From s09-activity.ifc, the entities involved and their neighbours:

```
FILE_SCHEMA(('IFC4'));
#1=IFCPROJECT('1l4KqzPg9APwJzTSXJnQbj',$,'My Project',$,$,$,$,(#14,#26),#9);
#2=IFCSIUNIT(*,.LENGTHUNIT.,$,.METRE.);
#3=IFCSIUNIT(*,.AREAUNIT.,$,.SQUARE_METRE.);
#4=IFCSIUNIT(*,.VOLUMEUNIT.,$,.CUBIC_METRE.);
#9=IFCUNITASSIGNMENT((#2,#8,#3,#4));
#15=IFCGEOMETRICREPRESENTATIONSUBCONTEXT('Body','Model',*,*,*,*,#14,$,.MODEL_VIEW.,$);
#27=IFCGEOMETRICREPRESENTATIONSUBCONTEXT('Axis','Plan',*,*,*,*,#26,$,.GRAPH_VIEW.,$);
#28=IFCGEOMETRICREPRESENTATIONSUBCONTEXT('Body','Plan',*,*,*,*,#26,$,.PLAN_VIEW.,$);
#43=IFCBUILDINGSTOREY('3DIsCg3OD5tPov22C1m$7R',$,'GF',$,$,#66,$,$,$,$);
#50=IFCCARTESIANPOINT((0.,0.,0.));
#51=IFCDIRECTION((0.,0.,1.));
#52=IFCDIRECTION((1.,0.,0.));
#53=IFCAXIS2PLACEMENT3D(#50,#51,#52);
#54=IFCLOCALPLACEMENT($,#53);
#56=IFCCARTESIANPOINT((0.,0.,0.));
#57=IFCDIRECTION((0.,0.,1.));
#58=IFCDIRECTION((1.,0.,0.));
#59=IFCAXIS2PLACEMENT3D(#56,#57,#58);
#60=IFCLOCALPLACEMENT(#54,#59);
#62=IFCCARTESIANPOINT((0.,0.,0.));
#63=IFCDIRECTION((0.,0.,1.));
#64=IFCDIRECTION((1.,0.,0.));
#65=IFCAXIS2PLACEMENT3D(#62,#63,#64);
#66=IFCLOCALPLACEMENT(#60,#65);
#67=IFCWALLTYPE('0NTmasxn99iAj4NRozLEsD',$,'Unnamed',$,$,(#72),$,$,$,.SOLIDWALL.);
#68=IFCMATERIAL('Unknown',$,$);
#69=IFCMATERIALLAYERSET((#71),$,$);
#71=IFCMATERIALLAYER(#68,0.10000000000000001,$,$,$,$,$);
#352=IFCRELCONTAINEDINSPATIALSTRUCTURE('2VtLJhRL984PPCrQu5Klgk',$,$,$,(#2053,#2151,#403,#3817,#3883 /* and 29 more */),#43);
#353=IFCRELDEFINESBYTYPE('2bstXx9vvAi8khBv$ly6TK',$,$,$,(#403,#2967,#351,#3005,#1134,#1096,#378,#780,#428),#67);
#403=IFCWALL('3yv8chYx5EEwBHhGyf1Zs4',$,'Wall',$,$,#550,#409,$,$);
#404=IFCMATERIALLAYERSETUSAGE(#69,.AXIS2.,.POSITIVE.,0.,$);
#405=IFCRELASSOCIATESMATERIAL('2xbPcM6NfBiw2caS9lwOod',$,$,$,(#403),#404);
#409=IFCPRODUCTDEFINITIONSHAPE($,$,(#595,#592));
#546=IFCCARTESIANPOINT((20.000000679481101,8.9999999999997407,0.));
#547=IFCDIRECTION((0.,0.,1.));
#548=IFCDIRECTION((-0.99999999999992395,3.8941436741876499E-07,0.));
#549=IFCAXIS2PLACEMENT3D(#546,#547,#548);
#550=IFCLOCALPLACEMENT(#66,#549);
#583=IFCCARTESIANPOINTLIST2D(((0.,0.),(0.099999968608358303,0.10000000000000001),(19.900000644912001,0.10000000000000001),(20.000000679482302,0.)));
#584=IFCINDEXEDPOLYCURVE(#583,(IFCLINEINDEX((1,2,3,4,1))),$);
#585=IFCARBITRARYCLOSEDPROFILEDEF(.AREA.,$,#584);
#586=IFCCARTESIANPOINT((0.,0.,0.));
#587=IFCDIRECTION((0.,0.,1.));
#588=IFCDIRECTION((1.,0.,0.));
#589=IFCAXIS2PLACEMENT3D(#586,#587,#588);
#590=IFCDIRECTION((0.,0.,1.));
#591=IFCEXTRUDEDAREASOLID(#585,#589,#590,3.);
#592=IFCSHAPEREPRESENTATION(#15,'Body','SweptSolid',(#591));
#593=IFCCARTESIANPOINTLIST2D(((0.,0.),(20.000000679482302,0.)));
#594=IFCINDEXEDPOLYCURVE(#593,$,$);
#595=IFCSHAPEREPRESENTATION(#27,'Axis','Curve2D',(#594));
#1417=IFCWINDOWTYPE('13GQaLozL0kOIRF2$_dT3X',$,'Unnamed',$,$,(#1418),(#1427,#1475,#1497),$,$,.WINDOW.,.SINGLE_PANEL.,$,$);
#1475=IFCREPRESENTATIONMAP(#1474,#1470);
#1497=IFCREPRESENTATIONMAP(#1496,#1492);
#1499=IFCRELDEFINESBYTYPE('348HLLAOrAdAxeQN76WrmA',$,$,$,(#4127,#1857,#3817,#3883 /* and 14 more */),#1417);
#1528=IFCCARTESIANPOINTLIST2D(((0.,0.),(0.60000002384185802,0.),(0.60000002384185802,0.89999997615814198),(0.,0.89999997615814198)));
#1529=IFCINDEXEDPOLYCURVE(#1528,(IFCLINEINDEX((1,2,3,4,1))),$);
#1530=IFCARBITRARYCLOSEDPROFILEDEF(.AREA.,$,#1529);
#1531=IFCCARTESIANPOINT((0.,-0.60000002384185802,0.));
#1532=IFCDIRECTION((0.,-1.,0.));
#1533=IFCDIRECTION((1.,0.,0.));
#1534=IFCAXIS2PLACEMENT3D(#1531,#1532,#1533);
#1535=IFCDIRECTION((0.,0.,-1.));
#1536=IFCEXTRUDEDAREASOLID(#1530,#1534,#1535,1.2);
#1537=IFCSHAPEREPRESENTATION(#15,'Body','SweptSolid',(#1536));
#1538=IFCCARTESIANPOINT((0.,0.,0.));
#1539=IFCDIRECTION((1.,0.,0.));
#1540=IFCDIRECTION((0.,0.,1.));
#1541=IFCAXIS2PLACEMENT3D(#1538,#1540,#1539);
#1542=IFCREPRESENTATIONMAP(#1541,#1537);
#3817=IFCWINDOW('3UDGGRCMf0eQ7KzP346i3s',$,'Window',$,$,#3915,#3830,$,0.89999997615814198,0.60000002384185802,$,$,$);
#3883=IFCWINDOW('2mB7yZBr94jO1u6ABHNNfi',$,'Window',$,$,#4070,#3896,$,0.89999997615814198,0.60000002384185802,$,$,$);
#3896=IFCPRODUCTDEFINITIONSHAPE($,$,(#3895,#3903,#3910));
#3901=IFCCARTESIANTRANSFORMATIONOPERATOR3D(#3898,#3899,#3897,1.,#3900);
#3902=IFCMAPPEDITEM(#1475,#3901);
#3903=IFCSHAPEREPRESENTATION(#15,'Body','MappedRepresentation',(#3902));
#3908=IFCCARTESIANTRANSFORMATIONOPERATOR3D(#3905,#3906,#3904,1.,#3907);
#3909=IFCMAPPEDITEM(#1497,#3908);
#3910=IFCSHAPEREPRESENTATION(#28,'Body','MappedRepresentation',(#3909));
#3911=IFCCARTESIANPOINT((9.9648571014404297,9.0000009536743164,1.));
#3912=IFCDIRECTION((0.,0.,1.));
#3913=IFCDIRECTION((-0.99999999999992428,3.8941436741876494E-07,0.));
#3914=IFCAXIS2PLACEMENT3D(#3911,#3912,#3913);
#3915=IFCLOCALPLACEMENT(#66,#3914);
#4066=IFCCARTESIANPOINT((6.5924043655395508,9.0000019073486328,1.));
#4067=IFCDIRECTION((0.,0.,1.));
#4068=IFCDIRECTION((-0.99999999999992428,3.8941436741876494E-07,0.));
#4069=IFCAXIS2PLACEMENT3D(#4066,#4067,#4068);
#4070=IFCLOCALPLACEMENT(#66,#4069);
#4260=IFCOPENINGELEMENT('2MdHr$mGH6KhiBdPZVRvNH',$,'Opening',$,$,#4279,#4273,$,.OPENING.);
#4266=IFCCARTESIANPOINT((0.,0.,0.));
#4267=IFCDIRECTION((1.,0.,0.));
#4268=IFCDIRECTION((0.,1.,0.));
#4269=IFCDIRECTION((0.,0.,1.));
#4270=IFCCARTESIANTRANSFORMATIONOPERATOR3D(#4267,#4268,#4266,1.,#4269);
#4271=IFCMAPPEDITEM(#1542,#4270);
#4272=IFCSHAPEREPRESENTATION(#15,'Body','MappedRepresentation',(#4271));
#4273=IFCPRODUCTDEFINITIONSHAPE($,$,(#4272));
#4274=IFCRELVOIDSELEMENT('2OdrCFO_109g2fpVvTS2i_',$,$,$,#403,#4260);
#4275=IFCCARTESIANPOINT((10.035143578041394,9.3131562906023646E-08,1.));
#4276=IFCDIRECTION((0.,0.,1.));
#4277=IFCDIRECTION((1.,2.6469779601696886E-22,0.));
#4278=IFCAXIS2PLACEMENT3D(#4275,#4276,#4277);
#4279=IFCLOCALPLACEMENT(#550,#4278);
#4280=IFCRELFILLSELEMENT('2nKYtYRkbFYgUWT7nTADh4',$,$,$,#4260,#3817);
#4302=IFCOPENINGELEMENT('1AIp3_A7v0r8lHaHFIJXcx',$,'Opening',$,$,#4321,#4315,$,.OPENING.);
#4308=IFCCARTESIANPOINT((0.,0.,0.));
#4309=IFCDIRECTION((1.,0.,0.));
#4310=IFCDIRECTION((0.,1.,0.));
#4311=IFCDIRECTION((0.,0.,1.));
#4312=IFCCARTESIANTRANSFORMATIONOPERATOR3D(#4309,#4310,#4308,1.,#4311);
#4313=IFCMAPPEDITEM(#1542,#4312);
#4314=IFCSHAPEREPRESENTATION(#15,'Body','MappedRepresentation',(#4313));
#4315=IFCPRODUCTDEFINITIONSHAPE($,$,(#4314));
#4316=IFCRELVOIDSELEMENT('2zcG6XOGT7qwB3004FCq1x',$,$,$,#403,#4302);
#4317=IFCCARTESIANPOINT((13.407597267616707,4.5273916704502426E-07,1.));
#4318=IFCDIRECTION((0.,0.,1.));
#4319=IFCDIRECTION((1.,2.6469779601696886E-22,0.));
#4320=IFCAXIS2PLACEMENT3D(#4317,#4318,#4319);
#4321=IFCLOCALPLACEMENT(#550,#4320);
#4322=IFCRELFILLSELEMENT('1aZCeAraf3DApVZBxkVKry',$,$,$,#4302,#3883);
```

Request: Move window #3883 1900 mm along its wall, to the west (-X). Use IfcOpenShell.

```python
import ifcopenshell
import ifcopenshell.api.geometry
import ifcopenshell.util.placement

model = ifcopenshell.open("s09-activity.ifc")

window = model.by_guid("2mB7yZBr94jO1u6ABHNNfi")
opening = window.FillsVoids[0].RelatingOpeningElement
wall = opening.VoidsElements[0].RelatingBuildingElement

wall_matrix = ifcopenshell.util.placement.get_local_placement(wall.ObjectPlacement)
shift = wall_matrix[:3, 0] * 1.9
before = ifcopenshell.util.placement.get_local_placement(window.ObjectPlacement)[:3, 3].copy()

# The window is not placed relative to its opening, so move both.
for product in (opening, window):
    matrix = ifcopenshell.util.placement.get_local_placement(product.ObjectPlacement)
    matrix[:3, 3] += shift
    ifcopenshell.api.geometry.edit_object_placement(model, product=product, matrix=matrix, is_si=False)

after = ifcopenshell.util.placement.get_local_placement(window.ObjectPlacement)[:3, 3]
print("window moved by", (after - before).round(3) + 0.0)

model.write("s09-activity_v2.ifc")
```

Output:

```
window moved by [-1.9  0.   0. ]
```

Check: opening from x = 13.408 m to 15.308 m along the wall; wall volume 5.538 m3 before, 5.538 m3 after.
